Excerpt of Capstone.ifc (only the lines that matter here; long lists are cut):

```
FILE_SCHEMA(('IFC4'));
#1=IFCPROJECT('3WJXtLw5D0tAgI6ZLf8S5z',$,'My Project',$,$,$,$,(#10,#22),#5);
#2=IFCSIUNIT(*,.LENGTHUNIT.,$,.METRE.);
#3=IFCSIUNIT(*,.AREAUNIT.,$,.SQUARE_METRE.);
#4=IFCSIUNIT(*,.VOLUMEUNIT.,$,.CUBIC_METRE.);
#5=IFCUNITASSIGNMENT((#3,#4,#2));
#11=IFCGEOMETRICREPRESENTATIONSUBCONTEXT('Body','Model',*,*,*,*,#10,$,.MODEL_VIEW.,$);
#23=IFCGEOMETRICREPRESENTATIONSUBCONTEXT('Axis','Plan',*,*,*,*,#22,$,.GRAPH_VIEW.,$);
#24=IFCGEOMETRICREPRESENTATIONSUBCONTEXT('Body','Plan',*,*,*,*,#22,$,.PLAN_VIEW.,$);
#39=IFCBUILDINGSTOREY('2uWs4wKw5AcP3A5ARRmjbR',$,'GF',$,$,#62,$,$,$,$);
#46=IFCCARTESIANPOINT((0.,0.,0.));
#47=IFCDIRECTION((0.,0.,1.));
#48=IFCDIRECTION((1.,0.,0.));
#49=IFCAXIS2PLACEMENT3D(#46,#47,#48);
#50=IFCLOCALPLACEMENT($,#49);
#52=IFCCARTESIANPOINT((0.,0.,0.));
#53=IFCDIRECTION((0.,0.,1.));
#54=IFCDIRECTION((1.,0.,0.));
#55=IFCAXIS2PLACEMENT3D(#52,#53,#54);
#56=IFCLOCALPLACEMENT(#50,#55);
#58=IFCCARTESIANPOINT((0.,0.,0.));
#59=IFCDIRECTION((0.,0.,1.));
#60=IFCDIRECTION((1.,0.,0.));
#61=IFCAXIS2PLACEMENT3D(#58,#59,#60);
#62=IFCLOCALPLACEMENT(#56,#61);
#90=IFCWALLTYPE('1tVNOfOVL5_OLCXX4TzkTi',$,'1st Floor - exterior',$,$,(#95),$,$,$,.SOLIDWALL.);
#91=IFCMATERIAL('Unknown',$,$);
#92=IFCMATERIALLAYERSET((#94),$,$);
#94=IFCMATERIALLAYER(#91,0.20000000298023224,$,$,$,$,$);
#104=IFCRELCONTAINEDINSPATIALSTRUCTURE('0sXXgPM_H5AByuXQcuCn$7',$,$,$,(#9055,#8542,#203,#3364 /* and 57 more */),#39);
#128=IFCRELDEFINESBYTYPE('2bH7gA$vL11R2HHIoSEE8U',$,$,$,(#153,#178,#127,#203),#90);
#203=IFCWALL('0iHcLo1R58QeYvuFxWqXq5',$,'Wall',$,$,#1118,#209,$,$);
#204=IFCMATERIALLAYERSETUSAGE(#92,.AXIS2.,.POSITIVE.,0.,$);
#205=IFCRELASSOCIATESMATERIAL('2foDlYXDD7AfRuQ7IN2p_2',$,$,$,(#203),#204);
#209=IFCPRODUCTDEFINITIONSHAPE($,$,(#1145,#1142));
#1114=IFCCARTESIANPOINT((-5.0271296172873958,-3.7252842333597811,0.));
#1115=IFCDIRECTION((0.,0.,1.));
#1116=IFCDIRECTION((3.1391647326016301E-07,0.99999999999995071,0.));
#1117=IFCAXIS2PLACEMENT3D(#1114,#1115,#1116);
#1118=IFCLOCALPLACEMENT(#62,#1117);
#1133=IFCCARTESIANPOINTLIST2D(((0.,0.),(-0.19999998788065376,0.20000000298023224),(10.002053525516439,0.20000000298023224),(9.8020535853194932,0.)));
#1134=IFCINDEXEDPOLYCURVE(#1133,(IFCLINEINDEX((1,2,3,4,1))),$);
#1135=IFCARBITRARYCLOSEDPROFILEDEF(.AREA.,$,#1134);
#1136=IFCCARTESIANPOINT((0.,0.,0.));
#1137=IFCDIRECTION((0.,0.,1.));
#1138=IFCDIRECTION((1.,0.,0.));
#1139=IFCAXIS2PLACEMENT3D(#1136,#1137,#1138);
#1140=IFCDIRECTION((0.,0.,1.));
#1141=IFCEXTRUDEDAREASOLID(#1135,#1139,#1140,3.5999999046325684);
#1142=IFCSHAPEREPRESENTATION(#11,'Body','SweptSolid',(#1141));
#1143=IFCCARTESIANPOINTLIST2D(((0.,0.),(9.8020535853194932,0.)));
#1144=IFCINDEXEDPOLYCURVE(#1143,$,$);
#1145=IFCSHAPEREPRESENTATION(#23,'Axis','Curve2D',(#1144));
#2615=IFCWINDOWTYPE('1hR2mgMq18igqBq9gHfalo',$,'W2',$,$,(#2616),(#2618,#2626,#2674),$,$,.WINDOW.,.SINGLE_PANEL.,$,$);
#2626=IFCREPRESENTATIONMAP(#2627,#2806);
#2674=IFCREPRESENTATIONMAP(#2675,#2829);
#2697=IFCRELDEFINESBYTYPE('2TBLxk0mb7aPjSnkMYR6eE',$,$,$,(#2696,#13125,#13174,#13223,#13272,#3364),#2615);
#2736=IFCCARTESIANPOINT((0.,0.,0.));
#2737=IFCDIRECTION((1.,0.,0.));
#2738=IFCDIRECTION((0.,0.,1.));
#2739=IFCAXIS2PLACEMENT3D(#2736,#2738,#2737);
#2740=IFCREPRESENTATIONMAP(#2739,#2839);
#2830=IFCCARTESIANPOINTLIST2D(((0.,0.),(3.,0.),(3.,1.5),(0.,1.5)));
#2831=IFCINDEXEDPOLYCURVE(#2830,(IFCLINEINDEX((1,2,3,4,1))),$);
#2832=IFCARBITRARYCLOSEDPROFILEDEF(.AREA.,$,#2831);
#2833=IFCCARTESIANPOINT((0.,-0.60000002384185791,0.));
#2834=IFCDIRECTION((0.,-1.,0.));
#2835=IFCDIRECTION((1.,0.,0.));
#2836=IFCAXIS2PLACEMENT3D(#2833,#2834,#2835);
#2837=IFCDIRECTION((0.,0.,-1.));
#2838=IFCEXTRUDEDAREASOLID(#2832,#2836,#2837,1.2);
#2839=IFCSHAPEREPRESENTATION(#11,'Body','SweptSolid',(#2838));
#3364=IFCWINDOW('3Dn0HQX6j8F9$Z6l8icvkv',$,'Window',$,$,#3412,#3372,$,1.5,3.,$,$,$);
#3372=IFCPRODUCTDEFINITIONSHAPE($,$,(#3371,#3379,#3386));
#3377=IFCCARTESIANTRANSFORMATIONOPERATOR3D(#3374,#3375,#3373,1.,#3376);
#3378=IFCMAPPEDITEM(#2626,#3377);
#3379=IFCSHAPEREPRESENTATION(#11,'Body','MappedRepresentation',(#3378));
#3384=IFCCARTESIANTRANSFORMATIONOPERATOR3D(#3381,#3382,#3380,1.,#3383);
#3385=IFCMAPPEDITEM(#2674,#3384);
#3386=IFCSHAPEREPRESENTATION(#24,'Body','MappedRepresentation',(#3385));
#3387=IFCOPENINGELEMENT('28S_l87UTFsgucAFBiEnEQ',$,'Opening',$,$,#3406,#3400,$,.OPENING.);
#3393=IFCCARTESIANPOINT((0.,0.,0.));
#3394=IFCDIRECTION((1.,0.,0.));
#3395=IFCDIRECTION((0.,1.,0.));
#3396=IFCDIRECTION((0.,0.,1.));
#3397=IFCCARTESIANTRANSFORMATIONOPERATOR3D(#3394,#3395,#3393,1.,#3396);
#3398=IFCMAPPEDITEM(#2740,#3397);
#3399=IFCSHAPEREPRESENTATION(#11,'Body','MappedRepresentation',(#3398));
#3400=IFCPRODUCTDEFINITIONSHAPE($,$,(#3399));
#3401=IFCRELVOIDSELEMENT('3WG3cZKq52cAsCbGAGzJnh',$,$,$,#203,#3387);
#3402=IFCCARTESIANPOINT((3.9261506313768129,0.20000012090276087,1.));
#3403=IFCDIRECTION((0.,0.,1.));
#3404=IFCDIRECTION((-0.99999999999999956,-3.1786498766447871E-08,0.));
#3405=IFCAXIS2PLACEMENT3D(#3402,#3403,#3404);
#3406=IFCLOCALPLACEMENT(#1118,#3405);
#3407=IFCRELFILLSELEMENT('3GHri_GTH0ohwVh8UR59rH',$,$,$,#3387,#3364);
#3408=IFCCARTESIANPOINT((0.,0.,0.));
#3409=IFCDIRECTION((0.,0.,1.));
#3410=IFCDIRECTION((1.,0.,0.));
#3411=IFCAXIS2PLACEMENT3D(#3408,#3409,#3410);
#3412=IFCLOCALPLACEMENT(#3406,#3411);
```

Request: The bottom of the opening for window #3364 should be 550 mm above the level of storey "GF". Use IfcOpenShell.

```python
import numpy as np
import ifcopenshell
import ifcopenshell.api.geometry
import ifcopenshell.geom
import ifcopenshell.util.element
import ifcopenshell.util.placement
import ifcopenshell.util.shape
import ifcopenshell.util.unit

model = ifcopenshell.open("Capstone.ifc")
unit_scale = ifcopenshell.util.unit.calculate_unit_scale(model)

window = model.by_guid("3Dn0HQX6j8F9$Z6l8icvkv")
opening = window.FillsVoids[0].RelatingOpeningElement
storey = ifcopenshell.util.element.get_container(window, ifc_class="IfcBuildingStorey")
level = ifcopenshell.util.placement.get_local_placement(storey.ObjectPlacement)[2, 3]

# The opening's origin need not be at the sill, so measure its lowest point.
shape = ifcopenshell.geom.create_shape(ifcopenshell.geom.settings(), opening)
bottom = ifcopenshell.util.shape.get_shape_bottom_elevation(shape, shape.geometry) / unit_scale
dz = level + 0.55 - bottom

shift = np.array([0.0, 0.0, dz])
# The window is placed relative to its opening, so it follows when the opening moves.
matrix = ifcopenshell.util.placement.get_local_placement(opening.ObjectPlacement)
matrix[:3, 3] += shift
ifcopenshell.api.geometry.edit_object_placement(
    model, product=opening, matrix=matrix, is_si=False, should_transform_children=True
)

print(f"moved by {dz * unit_scale:+.3f} m")

model.write("Capstone_updated.ifc")
```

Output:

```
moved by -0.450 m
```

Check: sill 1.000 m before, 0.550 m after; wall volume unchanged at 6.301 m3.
